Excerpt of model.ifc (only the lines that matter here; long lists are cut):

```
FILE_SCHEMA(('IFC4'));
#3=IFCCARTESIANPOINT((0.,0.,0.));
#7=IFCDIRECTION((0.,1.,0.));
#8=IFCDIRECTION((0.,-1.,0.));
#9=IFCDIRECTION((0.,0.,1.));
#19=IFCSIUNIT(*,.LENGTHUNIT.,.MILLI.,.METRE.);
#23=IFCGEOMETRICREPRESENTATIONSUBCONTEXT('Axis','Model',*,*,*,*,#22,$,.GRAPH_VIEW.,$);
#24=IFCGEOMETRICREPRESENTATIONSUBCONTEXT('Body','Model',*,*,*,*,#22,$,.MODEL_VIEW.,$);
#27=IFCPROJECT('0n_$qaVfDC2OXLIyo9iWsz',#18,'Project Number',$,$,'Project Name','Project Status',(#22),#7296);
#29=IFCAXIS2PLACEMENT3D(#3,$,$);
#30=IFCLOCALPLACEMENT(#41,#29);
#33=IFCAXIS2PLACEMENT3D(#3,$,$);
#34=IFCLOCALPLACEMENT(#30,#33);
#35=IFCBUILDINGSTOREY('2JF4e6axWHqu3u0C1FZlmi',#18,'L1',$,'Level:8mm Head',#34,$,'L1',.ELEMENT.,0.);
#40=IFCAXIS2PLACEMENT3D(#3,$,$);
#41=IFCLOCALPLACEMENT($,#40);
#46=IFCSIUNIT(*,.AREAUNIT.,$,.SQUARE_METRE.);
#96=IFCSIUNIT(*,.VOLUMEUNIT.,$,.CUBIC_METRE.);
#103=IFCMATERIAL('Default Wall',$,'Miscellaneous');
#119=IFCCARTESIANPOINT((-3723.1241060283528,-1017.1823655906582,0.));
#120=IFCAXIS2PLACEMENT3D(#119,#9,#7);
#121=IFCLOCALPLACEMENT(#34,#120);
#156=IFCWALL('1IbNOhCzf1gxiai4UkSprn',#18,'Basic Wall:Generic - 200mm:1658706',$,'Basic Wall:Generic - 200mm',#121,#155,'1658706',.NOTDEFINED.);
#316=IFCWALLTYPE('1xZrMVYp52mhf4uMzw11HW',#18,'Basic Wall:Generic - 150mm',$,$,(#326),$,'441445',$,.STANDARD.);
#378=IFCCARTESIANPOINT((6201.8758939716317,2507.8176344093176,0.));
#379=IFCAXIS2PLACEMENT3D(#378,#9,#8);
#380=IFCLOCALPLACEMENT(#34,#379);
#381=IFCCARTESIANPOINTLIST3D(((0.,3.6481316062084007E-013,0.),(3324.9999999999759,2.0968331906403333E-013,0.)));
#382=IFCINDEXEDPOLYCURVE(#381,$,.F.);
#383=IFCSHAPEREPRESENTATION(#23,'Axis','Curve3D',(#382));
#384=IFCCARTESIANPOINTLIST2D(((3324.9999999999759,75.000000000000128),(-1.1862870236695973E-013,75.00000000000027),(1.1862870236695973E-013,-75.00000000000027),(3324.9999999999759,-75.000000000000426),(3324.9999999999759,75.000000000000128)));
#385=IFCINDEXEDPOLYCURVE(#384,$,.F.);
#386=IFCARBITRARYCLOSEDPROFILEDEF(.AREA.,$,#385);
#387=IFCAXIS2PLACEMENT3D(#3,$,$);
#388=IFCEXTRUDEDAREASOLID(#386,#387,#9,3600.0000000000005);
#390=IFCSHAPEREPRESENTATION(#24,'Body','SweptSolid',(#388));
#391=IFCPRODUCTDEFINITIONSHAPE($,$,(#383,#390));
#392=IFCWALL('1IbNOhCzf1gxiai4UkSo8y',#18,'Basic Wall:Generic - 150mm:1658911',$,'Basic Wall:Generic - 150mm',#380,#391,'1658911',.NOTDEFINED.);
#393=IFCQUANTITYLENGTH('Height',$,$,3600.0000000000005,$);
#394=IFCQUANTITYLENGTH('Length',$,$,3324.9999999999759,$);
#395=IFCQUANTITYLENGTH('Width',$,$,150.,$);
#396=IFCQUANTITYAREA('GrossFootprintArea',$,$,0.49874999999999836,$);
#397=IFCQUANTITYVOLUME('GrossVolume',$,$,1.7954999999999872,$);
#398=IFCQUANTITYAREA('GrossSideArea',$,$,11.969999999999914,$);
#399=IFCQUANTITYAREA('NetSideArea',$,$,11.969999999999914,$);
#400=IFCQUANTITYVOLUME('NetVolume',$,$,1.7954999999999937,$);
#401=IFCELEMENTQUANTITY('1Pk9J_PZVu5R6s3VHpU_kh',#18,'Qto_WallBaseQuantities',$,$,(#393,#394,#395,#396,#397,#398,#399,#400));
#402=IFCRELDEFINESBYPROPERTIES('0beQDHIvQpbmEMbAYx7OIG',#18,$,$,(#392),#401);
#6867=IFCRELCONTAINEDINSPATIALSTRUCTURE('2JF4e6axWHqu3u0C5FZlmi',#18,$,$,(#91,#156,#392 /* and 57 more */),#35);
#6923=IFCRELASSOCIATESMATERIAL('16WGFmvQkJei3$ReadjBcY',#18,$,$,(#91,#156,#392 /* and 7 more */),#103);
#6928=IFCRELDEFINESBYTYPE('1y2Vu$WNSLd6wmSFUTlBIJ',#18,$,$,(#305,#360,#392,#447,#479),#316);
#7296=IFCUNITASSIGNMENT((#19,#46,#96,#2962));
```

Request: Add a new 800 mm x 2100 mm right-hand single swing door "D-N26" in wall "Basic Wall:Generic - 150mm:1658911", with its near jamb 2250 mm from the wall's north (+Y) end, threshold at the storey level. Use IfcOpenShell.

```python
import numpy as np
import ifcopenshell
import ifcopenshell.api.feature
import ifcopenshell.api.geometry
import ifcopenshell.api.pset
import ifcopenshell.api.root
import ifcopenshell.api.spatial
import ifcopenshell.geom
import ifcopenshell.util.element
import ifcopenshell.util.placement
import ifcopenshell.util.representation
import ifcopenshell.util.shape
import ifcopenshell.util.unit

model = ifcopenshell.open("model.ifc")
unit_scale = ifcopenshell.util.unit.calculate_unit_scale(model)
area_scale = ifcopenshell.util.unit.calculate_unit_scale(model, "AREAUNIT")
volume_scale = ifcopenshell.util.unit.calculate_unit_scale(model, "VOLUMEUNIT")
settings = ifcopenshell.geom.settings()


def volume(element):
    """Net volume in cubic metres, openings subtracted."""
    shape = ifcopenshell.geom.create_shape(settings, element)
    return ifcopenshell.util.shape.get_volume(shape.geometry)


wall = model.by_id(392)
storey = ifcopenshell.util.element.get_container(wall, ifc_class="IfcBuildingStorey")
context = ifcopenshell.util.representation.get_context(model, "Model", "Body", "MODEL_VIEW")
before = volume(wall)

width, height, from_end, sill = 0.8, 2.1, 2.25, 0.0  # metres

# The wall runs along its own X axis, and the end named is its -X end.
wall_shape = ifcopenshell.geom.create_shape(settings, wall)
x, y, z = ifcopenshell.util.shape.get_vertices(wall_shape.geometry).T
start = x.min() + from_end
face, thickness = float(y.min()), float(y.max() - y.min())
wall_matrix = ifcopenshell.util.placement.get_local_placement(wall.ObjectPlacement)
level = ifcopenshell.util.placement.get_local_placement(storey.ObjectPlacement)[2, 3]


def in_wall(x, y):
    """Placement at x, y metres in the wall's axes, at sill height."""
    matrix = wall_matrix.copy()
    matrix[:, 3] = wall_matrix @ np.array([x / unit_scale, y / unit_scale, 0.0, 1.0])
    matrix[2, 3] = level + sill / unit_scale
    return matrix


# Opening: a box that overshoots both wall faces by 50 mm.
opening = ifcopenshell.api.root.create_entity(model, ifc_class="IfcOpeningElement", predefined_type="OPENING")
box = ifcopenshell.api.geometry.add_wall_representation(
    model, context=context, length=width, height=height, thickness=thickness + 0.1
)
ifcopenshell.api.geometry.assign_representation(model, product=opening, representation=box)
ifcopenshell.api.geometry.edit_object_placement(model, product=opening, matrix=in_wall(start, face - 0.05), is_si=False)
ifcopenshell.api.feature.add_feature(model, feature=opening, element=wall)

door = ifcopenshell.api.root.create_entity(model, ifc_class="IfcDoor", name="D-N26", predefined_type="DOOR")
door.OverallWidth, door.OverallHeight = width / unit_scale, height / unit_scale
door.OperationType = "SINGLE_SWING_RIGHT"
body = ifcopenshell.api.geometry.add_door_representation(
    model,
    context=context,
    overall_width=door.OverallWidth,
    overall_height=door.OverallHeight,
    operation_type="SINGLE_SWING_RIGHT",
    lining_properties={"LiningDepth": thickness / unit_scale, "ThresholdDepth": thickness / unit_scale},
)
ifcopenshell.api.geometry.assign_representation(model, product=door, representation=body)
ifcopenshell.api.spatial.assign_container(model, products=[door], relating_structure=storey)
ifcopenshell.api.feature.add_filling(model, opening=opening, element=door)

# The lining spans the wall, so the door starts at the wall face.
ifcopenshell.api.geometry.edit_object_placement(model, product=door, matrix=in_wall(start, face), is_si=False)

after = volume(wall)

# Update the wall's stored quantities.
qto = model.by_id(ifcopenshell.util.element.get_pset(wall, "Qto_WallBaseQuantities", should_inherit=False)["id"])
ifcopenshell.api.pset.edit_qto(model, qto=qto, properties={
    "NetSideArea": after / thickness / area_scale,
    "NetVolume": after / volume_scale,
})

print(f"wall volume {before:.3f} -> {after:.3f} m3")

model.write("model_rev.ifc")
```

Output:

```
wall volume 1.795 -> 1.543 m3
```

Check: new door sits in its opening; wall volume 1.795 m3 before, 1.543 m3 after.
